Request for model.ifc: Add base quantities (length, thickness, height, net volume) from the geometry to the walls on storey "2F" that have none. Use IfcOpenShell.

First a look at what the model holds.

```python
import ifcopenshell
import ifcopenshell.util.element
import ifcopenshell.util.unit

model = ifcopenshell.open("model.ifc")
print(model.schema)
for unit_type in ("LENGTHUNIT", "AREAUNIT", "VOLUMEUNIT"):
    print(unit_type, ifcopenshell.util.unit.calculate_unit_scale(model, unit_type))
storey = next(s for s in model.by_type("IfcBuildingStorey") if s.Name == "2F")
walls = [e for e in ifcopenshell.util.element.get_decomposition(storey) if e.is_a("IfcWall")]
for e in sorted(walls, key=lambda e: e.id()):
    print(e.id(), e.is_a(), e.Name, list(ifcopenshell.util.element.get_psets(e, qtos_only=True)), sep=" | ")
```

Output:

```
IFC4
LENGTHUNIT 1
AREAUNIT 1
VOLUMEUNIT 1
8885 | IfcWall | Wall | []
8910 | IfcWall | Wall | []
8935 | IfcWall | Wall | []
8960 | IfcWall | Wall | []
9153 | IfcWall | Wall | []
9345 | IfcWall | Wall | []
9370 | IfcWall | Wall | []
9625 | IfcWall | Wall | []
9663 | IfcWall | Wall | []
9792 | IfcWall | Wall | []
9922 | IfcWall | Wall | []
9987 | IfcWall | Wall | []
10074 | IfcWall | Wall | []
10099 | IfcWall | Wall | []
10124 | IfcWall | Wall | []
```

```python
import ifcopenshell
import ifcopenshell.api.pset
import ifcopenshell.geom
import ifcopenshell.util.element
import ifcopenshell.util.shape
import ifcopenshell.util.unit

model = ifcopenshell.open("model.ifc")
unit_scale = ifcopenshell.util.unit.calculate_unit_scale(model)
volume_scale = ifcopenshell.util.unit.calculate_unit_scale(model, "VOLUMEUNIT")
settings = ifcopenshell.geom.settings()

storey = next(s for s in model.by_type("IfcBuildingStorey") if s.Name == "2F")
walls = [e for e in ifcopenshell.util.element.get_decomposition(storey) if e.is_a("IfcWall")]

for e in sorted(walls, key=lambda e: e.id()):
    if ifcopenshell.util.element.get_psets(e, qtos_only=True, should_inherit=False):
        continue
    # Geometry comes back in metres, in the element's own axes.
    shape = ifcopenshell.geom.create_shape(settings, e)
    values = {
        "Length": ifcopenshell.util.shape.get_x(shape.geometry) / unit_scale,
        "Width": ifcopenshell.util.shape.get_y(shape.geometry) / unit_scale,
        "Height": ifcopenshell.util.shape.get_z(shape.geometry) / unit_scale,
        "NetVolume": ifcopenshell.util.shape.get_volume(shape.geometry) / volume_scale,
    }
    qto = ifcopenshell.api.pset.add_qto(model, product=e, name="Qto_WallBaseQuantities")
    ifcopenshell.api.pset.edit_qto(model, qto=qto, properties=values)
    print(e.id(), {k: round(v, 3) for k, v in values.items()})

model.write("model_v2.ifc")
```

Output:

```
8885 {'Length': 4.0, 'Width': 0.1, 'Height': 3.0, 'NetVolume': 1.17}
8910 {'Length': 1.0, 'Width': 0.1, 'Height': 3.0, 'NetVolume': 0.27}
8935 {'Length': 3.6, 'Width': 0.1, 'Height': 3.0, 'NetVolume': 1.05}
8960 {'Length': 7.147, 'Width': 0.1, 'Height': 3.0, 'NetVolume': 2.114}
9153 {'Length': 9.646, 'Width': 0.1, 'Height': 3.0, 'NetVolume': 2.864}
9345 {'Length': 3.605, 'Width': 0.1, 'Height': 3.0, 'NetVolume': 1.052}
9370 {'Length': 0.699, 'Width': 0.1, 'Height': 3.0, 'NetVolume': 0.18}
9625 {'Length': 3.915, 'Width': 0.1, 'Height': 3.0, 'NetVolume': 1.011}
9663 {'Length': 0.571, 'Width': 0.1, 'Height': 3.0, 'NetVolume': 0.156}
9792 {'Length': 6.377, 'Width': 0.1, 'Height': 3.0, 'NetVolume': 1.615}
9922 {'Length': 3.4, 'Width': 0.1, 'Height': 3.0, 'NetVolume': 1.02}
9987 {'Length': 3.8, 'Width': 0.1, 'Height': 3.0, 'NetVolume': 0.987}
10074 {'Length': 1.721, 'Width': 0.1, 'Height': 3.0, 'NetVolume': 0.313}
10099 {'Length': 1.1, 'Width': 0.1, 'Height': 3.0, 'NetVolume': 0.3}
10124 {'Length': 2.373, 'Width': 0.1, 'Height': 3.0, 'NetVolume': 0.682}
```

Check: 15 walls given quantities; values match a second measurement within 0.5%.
